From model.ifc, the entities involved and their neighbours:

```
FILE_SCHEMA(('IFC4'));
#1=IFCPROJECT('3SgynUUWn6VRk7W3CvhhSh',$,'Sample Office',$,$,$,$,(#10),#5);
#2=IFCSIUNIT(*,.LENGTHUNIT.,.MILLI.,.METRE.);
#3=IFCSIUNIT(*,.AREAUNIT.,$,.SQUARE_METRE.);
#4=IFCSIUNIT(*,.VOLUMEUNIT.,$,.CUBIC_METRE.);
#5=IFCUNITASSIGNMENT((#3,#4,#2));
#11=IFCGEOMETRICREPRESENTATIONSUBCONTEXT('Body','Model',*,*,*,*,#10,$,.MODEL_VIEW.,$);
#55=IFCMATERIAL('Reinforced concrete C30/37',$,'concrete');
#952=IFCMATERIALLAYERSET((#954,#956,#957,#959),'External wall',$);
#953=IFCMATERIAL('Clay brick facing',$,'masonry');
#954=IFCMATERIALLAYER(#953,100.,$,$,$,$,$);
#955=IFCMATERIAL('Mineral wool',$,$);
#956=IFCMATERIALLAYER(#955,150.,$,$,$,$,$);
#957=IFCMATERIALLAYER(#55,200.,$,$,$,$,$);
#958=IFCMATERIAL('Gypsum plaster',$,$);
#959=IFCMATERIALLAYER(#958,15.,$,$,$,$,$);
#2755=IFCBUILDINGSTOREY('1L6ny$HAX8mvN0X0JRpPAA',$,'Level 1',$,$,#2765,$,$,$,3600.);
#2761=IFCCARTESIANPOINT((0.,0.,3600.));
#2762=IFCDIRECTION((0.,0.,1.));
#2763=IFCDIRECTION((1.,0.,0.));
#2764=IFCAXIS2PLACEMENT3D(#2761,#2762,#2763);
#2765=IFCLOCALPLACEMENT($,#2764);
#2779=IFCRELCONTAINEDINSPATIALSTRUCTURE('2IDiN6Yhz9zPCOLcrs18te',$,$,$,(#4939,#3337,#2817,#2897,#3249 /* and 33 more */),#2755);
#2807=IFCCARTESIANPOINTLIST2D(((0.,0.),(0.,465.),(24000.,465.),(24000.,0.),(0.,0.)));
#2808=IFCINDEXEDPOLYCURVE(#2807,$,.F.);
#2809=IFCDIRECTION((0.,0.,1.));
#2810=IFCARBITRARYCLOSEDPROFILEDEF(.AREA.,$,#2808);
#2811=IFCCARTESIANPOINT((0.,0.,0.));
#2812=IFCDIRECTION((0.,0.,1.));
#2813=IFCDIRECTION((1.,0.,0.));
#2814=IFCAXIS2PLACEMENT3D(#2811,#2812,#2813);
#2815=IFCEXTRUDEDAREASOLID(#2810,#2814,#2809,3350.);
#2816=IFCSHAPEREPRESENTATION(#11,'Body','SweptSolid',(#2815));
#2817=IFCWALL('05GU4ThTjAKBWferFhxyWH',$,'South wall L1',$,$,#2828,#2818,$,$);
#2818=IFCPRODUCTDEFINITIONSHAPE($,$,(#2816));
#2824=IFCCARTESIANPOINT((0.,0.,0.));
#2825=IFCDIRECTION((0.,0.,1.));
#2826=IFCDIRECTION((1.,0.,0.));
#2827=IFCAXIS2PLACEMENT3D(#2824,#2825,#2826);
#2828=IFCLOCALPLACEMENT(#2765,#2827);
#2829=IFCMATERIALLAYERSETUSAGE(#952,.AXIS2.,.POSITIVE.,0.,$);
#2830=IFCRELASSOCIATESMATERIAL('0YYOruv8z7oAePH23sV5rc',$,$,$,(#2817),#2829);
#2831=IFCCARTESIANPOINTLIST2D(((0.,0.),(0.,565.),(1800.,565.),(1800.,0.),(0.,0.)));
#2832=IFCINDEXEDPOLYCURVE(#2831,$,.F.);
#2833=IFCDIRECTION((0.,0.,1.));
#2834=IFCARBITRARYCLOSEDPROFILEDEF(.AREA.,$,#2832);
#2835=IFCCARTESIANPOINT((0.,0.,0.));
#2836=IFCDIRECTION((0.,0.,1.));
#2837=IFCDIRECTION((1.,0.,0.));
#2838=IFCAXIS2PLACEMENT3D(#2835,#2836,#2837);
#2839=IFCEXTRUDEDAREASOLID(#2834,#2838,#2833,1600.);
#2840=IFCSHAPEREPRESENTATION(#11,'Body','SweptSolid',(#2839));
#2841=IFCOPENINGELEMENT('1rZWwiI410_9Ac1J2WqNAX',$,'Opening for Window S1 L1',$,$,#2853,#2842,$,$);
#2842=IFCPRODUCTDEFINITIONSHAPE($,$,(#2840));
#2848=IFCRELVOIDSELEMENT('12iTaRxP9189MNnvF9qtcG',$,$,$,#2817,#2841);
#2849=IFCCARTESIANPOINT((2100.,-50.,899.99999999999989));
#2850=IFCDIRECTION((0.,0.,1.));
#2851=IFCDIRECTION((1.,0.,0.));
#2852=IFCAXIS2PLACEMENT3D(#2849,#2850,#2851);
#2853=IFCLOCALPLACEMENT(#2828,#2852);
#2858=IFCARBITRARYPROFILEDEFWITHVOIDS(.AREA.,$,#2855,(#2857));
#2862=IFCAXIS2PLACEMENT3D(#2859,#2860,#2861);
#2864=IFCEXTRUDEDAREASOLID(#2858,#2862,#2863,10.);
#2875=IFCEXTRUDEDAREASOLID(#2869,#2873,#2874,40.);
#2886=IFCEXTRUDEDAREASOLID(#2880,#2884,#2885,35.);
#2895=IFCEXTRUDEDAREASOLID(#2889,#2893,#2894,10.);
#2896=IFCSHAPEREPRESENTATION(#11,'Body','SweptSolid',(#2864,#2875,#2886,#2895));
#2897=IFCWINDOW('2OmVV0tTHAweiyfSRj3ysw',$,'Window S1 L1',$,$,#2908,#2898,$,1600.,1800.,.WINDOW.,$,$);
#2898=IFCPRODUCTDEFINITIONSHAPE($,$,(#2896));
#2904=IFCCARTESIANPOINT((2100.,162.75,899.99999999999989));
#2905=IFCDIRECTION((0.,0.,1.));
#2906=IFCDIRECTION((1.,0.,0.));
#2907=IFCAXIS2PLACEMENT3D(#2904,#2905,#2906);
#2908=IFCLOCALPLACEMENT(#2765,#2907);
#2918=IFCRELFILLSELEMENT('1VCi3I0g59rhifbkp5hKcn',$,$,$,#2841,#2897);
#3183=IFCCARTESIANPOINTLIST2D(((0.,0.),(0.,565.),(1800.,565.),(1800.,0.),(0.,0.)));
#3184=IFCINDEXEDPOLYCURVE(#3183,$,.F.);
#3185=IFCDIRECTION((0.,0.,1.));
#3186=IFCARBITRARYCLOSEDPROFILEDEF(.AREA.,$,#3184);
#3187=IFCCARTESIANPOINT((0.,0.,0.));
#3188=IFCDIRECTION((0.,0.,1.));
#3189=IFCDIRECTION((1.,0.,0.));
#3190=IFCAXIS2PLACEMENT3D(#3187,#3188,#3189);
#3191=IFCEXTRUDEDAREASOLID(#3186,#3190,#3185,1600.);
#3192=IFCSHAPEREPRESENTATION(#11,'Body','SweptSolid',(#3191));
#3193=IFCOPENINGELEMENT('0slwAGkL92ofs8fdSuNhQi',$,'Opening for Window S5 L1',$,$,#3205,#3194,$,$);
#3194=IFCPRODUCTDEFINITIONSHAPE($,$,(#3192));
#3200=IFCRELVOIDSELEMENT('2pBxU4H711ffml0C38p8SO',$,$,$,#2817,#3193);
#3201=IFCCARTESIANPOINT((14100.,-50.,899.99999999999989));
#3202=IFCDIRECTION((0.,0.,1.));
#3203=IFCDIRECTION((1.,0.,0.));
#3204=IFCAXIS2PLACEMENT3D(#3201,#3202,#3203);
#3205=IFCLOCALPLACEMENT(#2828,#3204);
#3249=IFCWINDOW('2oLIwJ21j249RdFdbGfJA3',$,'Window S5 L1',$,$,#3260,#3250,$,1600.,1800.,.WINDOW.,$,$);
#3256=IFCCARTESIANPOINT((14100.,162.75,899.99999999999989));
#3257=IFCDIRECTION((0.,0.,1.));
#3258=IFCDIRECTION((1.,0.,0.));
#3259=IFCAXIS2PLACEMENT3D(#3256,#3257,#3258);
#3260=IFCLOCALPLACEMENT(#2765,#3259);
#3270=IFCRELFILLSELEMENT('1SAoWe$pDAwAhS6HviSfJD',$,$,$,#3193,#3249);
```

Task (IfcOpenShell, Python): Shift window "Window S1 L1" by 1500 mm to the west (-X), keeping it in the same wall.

```python
import ifcopenshell
import ifcopenshell.api.geometry
import ifcopenshell.util.placement

model = ifcopenshell.open("model.ifc")

window = model.by_guid("2OmVV0tTHAweiyfSRj3ysw")
opening = window.FillsVoids[0].RelatingOpeningElement
wall = opening.VoidsElements[0].RelatingBuildingElement

wall_matrix = ifcopenshell.util.placement.get_local_placement(wall.ObjectPlacement)
shift = wall_matrix[:3, 0] * -1500.0
before = ifcopenshell.util.placement.get_local_placement(window.ObjectPlacement)[:3, 3].copy()

# The window is not placed relative to its opening, so move both.
for product in (opening, window):
    matrix = ifcopenshell.util.placement.get_local_placement(product.ObjectPlacement)
    matrix[:3, 3] += shift
    ifcopenshell.api.geometry.edit_object_placement(model, product=product, matrix=matrix, is_si=False)

after = ifcopenshell.util.placement.get_local_placement(window.ObjectPlacement)[:3, 3]
print("window moved by", (after - before).round(3) + 0.0)

model.write("model_rev.ifc")
```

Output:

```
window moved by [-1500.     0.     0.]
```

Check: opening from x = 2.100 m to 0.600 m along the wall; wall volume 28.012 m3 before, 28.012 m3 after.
